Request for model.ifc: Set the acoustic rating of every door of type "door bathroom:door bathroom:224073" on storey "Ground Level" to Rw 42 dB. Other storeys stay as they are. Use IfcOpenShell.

First a look at what the model holds.

```python
import ifcopenshell
import ifcopenshell.util.element

model = ifcopenshell.open("model.ifc")
print(model.schema)
storey = next(s for s in model.by_type("IfcBuildingStorey") if s.Name == "Ground Level")
doors = [e for e in ifcopenshell.util.element.get_decomposition(storey) if e.is_a("IfcDoor")]
seen = {}
for e in doors:
    element_type = ifcopenshell.util.element.get_type(e)
    key = (element_type.Name if element_type != e and element_type else None, ifcopenshell.util.element.get_pset(e, "Pset_DoorCommon", "AcousticRating"))
    seen[key] = seen.get(key, 0) + 1
for (name, value), count in sorted(seen.items(), key=str):
    print(count, "x", name, "|", value)
```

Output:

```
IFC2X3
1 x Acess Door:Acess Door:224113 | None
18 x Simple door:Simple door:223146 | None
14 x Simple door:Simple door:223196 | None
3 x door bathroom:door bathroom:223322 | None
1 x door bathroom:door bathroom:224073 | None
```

```python
import ifcopenshell
import ifcopenshell.api.pset
import ifcopenshell.util.element

model = ifcopenshell.open("model.ifc")

storey = next(s for s in model.by_type("IfcBuildingStorey") if s.Name == "Ground Level")
doors = [e for e in ifcopenshell.util.element.get_decomposition(storey) if e.is_a("IfcDoor")]

count = 0
for e in doors:
    element_type = ifcopenshell.util.element.get_type(e)
    if element_type in (None, e) or element_type.Name != "door bathroom:door bathroom:224073":
        continue
    # add_pset returns the element's existing set when there is one.
    pset = ifcopenshell.api.pset.add_pset(model, product=e, name="Pset_DoorCommon")
    ifcopenshell.api.pset.edit_pset(model, pset=pset, properties={"AcousticRating": "Rw 42 dB"})
    count += 1

print(count, "doors updated")

model.write("model_updated.ifc")
```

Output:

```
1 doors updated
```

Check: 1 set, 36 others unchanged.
